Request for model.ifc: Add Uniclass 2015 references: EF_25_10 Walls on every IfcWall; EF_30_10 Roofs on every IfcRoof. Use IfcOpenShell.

First a look at what the model holds.

```python
import ifcopenshell

model = ifcopenshell.open("model.ifc")
print(model.schema)
print("classifications:", [c.Name for c in model.by_type("IfcClassification")])
for ifc_class in ("IfcDoor", "IfcRoof", "IfcStair", "IfcWall", "IfcWindow"):
    print(ifc_class, len(model.by_type(ifc_class)))
```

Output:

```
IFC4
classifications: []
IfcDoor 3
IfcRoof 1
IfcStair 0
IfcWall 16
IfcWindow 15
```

```python
import ifcopenshell
import ifcopenshell.api.classification

model = ifcopenshell.open("model.ifc")

system = ifcopenshell.api.classification.add_classification(model, classification="Uniclass 2015")

codes = {
    "IfcWall": ("EF_25_10", "Walls"),
    "IfcRoof": ("EF_30_10", "Roofs"),
}
for ifc_class, (code, name) in codes.items():
    products = model.by_type(ifc_class)
    ifcopenshell.api.classification.add_reference(
        model, products=products, classification=system, identification=code, name=name
    )
    print(code, len(products))

model.write("model_updated.ifc")
```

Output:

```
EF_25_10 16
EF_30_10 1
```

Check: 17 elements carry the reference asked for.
